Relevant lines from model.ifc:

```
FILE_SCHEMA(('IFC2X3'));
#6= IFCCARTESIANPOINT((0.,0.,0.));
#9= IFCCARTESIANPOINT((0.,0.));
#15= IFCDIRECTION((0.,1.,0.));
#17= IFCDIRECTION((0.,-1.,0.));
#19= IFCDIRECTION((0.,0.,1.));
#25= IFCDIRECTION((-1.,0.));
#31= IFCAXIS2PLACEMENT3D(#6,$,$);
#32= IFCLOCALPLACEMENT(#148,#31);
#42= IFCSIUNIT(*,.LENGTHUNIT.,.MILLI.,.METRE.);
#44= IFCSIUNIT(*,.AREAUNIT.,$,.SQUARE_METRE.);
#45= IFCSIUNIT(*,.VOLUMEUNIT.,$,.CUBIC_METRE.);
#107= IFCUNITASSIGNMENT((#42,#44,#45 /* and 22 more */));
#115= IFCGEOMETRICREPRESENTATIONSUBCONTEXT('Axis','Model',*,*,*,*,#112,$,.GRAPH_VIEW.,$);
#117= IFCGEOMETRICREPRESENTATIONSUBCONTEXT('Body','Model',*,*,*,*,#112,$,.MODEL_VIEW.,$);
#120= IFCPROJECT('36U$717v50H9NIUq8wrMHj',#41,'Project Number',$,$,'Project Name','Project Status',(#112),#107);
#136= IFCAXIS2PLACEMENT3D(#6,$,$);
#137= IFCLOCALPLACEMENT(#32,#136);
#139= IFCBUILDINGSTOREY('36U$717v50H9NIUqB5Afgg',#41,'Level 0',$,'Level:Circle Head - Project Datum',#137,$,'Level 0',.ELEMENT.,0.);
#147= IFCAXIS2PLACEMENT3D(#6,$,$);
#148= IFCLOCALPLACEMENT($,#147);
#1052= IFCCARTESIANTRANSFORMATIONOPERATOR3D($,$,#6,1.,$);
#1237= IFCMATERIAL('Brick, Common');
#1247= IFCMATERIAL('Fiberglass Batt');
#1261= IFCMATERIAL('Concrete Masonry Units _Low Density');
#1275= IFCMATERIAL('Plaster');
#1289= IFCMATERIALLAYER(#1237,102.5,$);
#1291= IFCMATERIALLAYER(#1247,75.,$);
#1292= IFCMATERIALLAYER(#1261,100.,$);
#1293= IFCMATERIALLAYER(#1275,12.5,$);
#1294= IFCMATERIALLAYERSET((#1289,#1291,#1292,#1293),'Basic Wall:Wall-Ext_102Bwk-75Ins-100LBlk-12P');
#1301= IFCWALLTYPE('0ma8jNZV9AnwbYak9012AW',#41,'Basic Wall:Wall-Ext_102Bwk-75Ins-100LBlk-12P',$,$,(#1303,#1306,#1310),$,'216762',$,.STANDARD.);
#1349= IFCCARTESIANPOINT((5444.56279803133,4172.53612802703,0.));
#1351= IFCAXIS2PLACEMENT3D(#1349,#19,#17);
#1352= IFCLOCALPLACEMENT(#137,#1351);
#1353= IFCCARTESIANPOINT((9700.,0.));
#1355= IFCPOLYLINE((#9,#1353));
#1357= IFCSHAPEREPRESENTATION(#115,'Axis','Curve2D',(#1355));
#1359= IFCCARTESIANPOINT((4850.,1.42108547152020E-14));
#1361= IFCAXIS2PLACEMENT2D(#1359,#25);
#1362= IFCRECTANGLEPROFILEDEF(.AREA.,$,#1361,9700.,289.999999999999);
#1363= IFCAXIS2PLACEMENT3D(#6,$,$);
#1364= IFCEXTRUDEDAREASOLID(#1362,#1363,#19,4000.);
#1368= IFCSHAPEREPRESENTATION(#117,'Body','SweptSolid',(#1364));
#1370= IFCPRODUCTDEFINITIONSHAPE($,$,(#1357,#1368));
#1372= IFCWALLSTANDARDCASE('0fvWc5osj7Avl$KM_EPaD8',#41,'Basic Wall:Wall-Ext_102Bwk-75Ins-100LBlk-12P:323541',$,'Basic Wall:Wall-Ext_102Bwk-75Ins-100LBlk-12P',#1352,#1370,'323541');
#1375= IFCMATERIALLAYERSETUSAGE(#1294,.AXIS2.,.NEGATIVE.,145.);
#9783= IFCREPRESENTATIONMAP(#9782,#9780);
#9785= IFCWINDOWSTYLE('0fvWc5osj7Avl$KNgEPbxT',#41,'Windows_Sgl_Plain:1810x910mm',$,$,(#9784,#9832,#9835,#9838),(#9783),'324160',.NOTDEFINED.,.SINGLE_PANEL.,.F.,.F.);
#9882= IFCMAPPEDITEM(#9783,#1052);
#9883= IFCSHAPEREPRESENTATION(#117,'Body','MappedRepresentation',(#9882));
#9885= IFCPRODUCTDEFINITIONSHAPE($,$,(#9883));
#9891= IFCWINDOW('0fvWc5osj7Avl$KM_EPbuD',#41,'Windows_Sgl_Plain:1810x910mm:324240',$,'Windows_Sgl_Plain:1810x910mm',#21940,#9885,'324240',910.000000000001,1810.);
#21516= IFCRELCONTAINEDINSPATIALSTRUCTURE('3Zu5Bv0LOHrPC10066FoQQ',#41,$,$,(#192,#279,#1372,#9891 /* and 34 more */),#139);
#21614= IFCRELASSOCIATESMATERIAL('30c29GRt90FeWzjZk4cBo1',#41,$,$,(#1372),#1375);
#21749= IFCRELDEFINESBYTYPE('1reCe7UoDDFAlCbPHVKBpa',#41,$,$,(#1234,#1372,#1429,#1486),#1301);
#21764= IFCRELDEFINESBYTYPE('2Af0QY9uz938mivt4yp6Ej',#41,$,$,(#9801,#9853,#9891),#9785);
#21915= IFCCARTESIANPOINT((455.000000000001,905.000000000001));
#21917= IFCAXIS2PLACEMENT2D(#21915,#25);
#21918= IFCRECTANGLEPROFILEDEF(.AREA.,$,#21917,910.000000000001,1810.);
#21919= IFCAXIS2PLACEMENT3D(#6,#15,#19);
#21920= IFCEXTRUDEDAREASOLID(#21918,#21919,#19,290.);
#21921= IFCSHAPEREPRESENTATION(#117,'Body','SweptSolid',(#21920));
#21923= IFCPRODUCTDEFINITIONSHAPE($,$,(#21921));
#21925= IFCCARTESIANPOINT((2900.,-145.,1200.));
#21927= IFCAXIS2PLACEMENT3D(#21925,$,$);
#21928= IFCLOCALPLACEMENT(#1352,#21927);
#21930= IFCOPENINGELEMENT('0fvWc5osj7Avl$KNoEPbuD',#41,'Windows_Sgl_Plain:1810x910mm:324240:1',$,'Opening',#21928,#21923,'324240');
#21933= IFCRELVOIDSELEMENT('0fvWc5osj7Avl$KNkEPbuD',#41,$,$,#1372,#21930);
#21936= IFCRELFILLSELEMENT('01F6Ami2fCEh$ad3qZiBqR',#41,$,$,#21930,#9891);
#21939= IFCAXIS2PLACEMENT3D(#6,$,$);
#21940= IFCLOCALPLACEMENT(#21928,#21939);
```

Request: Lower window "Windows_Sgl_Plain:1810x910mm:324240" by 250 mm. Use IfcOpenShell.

```python
import numpy as np
import ifcopenshell
import ifcopenshell.api.geometry
import ifcopenshell.util.placement
import ifcopenshell.util.unit

model = ifcopenshell.open("model.ifc")
unit_scale = ifcopenshell.util.unit.calculate_unit_scale(model)

window = model.by_guid("0fvWc5osj7Avl$KM_EPbuD")
opening = window.FillsVoids[0].RelatingOpeningElement
dz = -250.0

shift = np.array([0.0, 0.0, dz])
# The window is placed relative to its opening, so it follows when the opening moves.
matrix = ifcopenshell.util.placement.get_local_placement(opening.ObjectPlacement)
matrix[:3, 3] += shift
ifcopenshell.api.geometry.edit_object_placement(
    model, product=opening, matrix=matrix, is_si=False, should_transform_children=True
)

print(f"moved by {dz * unit_scale:+.3f} m")

model.write("model-out.ifc")
```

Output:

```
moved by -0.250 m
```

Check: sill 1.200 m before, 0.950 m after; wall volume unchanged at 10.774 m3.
